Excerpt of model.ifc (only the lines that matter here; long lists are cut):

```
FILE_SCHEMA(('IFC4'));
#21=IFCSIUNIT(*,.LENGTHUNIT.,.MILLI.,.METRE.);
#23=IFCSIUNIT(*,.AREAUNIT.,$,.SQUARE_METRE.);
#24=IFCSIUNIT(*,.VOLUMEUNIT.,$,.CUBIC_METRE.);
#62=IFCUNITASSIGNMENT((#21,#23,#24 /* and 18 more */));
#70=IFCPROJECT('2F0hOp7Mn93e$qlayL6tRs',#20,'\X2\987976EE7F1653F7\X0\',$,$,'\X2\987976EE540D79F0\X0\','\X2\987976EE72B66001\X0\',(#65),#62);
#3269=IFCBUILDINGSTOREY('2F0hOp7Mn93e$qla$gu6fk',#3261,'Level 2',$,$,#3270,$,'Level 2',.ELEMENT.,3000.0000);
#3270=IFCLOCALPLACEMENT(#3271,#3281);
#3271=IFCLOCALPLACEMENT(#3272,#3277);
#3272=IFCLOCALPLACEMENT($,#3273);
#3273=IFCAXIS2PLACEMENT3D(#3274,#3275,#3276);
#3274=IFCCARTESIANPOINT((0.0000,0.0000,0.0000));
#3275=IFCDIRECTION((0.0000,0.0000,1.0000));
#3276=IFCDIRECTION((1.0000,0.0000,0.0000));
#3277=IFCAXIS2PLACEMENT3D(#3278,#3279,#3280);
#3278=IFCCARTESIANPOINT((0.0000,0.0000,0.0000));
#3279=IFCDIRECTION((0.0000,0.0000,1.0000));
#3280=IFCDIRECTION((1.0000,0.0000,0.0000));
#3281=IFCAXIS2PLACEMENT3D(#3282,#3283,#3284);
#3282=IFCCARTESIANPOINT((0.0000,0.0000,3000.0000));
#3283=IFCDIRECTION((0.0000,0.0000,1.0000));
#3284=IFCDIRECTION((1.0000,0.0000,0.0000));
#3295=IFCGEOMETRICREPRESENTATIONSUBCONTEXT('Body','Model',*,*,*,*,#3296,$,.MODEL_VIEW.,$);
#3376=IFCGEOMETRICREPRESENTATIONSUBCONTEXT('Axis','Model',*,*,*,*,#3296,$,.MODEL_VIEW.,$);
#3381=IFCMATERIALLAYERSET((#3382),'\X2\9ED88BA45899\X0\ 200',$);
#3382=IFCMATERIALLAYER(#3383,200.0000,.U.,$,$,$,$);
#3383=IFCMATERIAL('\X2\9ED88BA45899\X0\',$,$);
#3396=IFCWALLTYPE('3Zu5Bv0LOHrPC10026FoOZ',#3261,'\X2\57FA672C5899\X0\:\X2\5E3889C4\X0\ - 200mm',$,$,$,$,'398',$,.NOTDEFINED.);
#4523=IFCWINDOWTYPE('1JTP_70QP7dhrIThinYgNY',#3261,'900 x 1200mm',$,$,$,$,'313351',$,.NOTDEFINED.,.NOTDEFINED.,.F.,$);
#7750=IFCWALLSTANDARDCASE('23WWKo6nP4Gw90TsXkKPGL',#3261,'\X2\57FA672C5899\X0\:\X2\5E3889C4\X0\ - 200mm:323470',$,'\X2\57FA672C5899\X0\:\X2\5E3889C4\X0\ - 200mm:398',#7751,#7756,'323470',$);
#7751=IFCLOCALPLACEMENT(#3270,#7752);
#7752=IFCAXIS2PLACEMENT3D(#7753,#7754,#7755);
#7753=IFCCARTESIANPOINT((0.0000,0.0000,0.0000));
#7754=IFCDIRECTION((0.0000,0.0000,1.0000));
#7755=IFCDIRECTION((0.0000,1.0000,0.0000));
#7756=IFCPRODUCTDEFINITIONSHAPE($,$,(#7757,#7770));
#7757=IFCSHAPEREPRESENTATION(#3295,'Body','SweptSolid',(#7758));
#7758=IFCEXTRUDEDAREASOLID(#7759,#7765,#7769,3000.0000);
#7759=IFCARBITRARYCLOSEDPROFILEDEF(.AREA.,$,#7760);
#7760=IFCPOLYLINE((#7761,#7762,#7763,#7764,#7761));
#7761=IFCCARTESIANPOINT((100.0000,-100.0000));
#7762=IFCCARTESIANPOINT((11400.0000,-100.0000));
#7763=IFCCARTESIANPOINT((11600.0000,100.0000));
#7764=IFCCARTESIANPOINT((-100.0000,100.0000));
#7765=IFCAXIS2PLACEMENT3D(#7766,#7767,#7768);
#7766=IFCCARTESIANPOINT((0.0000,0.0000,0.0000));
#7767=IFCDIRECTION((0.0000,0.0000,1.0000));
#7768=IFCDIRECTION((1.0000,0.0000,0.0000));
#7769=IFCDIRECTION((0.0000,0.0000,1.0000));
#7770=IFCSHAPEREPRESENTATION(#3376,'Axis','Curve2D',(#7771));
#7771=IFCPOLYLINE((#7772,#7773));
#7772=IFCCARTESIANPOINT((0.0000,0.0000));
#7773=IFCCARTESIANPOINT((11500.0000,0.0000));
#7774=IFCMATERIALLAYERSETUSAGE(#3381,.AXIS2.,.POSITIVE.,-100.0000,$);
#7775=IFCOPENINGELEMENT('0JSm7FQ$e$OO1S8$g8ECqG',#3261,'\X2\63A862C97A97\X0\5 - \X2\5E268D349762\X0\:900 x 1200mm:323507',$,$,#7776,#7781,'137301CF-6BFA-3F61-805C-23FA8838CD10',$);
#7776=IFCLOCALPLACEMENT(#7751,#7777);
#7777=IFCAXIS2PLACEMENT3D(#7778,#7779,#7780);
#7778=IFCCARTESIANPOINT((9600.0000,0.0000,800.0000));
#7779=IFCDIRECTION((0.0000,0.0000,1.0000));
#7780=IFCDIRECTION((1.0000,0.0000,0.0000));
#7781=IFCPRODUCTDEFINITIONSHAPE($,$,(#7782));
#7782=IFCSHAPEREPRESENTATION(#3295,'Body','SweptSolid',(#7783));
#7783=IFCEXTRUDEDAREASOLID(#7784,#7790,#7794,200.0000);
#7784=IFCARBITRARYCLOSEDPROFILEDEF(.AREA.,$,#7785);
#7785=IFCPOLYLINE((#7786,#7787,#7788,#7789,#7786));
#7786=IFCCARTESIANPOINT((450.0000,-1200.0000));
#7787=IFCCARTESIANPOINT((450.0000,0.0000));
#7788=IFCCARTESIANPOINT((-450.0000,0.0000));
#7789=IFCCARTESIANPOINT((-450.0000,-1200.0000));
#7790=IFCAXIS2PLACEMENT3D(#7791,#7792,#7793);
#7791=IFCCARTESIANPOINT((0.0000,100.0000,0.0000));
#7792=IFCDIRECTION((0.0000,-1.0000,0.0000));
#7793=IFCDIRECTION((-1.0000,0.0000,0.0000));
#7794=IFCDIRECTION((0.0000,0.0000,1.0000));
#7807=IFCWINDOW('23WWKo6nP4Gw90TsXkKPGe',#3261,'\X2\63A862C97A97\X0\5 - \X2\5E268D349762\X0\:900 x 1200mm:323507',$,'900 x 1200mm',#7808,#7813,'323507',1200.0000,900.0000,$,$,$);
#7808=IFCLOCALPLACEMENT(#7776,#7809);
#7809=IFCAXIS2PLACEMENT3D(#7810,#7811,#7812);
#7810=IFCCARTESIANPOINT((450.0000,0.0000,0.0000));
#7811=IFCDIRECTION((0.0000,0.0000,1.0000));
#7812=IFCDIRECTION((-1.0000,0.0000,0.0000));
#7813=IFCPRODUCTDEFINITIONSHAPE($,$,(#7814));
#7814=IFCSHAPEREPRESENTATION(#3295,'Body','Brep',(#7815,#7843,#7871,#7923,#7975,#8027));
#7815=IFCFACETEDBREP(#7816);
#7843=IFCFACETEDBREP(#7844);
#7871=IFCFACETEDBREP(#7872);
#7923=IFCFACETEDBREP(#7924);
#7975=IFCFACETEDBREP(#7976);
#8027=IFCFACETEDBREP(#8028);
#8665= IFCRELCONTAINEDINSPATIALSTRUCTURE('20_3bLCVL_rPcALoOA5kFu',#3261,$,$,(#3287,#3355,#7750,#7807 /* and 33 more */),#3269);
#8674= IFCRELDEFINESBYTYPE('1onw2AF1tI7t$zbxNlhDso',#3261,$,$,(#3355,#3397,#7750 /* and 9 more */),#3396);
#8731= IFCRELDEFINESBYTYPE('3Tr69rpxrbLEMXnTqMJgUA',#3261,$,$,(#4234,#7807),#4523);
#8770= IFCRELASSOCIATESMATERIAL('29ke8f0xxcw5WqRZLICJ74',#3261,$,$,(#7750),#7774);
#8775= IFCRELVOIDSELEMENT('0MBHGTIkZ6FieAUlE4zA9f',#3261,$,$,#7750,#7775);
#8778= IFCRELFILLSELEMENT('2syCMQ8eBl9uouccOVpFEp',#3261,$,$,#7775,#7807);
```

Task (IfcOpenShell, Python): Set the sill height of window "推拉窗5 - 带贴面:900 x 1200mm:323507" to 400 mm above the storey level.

```python
import numpy as np
import ifcopenshell
import ifcopenshell.api.geometry
import ifcopenshell.geom
import ifcopenshell.util.element
import ifcopenshell.util.placement
import ifcopenshell.util.shape
import ifcopenshell.util.unit

model = ifcopenshell.open("model.ifc")
unit_scale = ifcopenshell.util.unit.calculate_unit_scale(model)

window = model.by_guid("23WWKo6nP4Gw90TsXkKPGe")
opening = window.FillsVoids[0].RelatingOpeningElement
storey = ifcopenshell.util.element.get_container(window, ifc_class="IfcBuildingStorey")
level = ifcopenshell.util.placement.get_local_placement(storey.ObjectPlacement)[2, 3]

# The opening's origin need not be at the sill, so measure its lowest point.
shape = ifcopenshell.geom.create_shape(ifcopenshell.geom.settings(), opening)
bottom = ifcopenshell.util.shape.get_shape_bottom_elevation(shape, shape.geometry) / unit_scale
dz = level + 400.0 - bottom

shift = np.array([0.0, 0.0, dz])
# The window is placed relative to its opening, so it follows when the opening moves.
matrix = ifcopenshell.util.placement.get_local_placement(opening.ObjectPlacement)
matrix[:3, 3] += shift
ifcopenshell.api.geometry.edit_object_placement(
    model, product=opening, matrix=matrix, is_si=False, should_transform_children=True
)

print(f"moved by {dz * unit_scale:+.3f} m")

model.write("model-out.ifc")
```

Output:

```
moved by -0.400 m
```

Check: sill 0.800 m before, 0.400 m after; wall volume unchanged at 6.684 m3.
